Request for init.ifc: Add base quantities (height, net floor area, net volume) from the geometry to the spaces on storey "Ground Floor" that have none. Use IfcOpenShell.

First a look at what the model holds.

```python
import ifcopenshell
import ifcopenshell.util.element
import ifcopenshell.util.unit

model = ifcopenshell.open("init.ifc")
print(model.schema)
for unit_type in ("LENGTHUNIT", "AREAUNIT", "VOLUMEUNIT"):
    print(unit_type, ifcopenshell.util.unit.calculate_unit_scale(model, unit_type))
storey = next(s for s in model.by_type("IfcBuildingStorey") if s.Name == "Ground Floor")
spaces = [e for e in ifcopenshell.util.element.get_decomposition(storey) if e.is_a("IfcSpace")]
for e in sorted(spaces, key=lambda e: e.id()):
    print(e.id(), e.is_a(), e.Name, list(ifcopenshell.util.element.get_psets(e, qtos_only=True)), sep=" | ")
```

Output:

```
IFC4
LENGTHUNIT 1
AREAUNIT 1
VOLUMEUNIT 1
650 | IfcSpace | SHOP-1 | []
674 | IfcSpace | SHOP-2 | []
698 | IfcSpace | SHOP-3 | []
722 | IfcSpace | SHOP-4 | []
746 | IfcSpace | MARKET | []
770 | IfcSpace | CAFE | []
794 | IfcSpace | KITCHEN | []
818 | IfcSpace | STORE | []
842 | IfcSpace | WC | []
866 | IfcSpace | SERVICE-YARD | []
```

```python
import ifcopenshell
import ifcopenshell.api.pset
import ifcopenshell.geom
import ifcopenshell.util.element
import ifcopenshell.util.shape
import ifcopenshell.util.unit

model = ifcopenshell.open("init.ifc")
unit_scale = ifcopenshell.util.unit.calculate_unit_scale(model)
area_scale = ifcopenshell.util.unit.calculate_unit_scale(model, "AREAUNIT")
volume_scale = ifcopenshell.util.unit.calculate_unit_scale(model, "VOLUMEUNIT")
settings = ifcopenshell.geom.settings()

storey = next(s for s in model.by_type("IfcBuildingStorey") if s.Name == "Ground Floor")
spaces = [e for e in ifcopenshell.util.element.get_decomposition(storey) if e.is_a("IfcSpace")]

for e in sorted(spaces, key=lambda e: e.id()):
    if ifcopenshell.util.element.get_psets(e, qtos_only=True, should_inherit=False):
        continue
    # Geometry comes back in metres, in the element's own axes.
    shape = ifcopenshell.geom.create_shape(settings, e)
    values = {
        "Height": ifcopenshell.util.shape.get_z(shape.geometry) / unit_scale,
        "NetFloorArea": ifcopenshell.util.shape.get_footprint_area(shape.geometry) / area_scale,
        "NetVolume": ifcopenshell.util.shape.get_volume(shape.geometry) / volume_scale,
    }
    qto = ifcopenshell.api.pset.add_qto(model, product=e, name="Qto_SpaceBaseQuantities")
    ifcopenshell.api.pset.edit_qto(model, qto=qto, properties=values)
    print(e.id(), {k: round(v, 3) for k, v in values.items()})

model.write("init-out.ifc")
```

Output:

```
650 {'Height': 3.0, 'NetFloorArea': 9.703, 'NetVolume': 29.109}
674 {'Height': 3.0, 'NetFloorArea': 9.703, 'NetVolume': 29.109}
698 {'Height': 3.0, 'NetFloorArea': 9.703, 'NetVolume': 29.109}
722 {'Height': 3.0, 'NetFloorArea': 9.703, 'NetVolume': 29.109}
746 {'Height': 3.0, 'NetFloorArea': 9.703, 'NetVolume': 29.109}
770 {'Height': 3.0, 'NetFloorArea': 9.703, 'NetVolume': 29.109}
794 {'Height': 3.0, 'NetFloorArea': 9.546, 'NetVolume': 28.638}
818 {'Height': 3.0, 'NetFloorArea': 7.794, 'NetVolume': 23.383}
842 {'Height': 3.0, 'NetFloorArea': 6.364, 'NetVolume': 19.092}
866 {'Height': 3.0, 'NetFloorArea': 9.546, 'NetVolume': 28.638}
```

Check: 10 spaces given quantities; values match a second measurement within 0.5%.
